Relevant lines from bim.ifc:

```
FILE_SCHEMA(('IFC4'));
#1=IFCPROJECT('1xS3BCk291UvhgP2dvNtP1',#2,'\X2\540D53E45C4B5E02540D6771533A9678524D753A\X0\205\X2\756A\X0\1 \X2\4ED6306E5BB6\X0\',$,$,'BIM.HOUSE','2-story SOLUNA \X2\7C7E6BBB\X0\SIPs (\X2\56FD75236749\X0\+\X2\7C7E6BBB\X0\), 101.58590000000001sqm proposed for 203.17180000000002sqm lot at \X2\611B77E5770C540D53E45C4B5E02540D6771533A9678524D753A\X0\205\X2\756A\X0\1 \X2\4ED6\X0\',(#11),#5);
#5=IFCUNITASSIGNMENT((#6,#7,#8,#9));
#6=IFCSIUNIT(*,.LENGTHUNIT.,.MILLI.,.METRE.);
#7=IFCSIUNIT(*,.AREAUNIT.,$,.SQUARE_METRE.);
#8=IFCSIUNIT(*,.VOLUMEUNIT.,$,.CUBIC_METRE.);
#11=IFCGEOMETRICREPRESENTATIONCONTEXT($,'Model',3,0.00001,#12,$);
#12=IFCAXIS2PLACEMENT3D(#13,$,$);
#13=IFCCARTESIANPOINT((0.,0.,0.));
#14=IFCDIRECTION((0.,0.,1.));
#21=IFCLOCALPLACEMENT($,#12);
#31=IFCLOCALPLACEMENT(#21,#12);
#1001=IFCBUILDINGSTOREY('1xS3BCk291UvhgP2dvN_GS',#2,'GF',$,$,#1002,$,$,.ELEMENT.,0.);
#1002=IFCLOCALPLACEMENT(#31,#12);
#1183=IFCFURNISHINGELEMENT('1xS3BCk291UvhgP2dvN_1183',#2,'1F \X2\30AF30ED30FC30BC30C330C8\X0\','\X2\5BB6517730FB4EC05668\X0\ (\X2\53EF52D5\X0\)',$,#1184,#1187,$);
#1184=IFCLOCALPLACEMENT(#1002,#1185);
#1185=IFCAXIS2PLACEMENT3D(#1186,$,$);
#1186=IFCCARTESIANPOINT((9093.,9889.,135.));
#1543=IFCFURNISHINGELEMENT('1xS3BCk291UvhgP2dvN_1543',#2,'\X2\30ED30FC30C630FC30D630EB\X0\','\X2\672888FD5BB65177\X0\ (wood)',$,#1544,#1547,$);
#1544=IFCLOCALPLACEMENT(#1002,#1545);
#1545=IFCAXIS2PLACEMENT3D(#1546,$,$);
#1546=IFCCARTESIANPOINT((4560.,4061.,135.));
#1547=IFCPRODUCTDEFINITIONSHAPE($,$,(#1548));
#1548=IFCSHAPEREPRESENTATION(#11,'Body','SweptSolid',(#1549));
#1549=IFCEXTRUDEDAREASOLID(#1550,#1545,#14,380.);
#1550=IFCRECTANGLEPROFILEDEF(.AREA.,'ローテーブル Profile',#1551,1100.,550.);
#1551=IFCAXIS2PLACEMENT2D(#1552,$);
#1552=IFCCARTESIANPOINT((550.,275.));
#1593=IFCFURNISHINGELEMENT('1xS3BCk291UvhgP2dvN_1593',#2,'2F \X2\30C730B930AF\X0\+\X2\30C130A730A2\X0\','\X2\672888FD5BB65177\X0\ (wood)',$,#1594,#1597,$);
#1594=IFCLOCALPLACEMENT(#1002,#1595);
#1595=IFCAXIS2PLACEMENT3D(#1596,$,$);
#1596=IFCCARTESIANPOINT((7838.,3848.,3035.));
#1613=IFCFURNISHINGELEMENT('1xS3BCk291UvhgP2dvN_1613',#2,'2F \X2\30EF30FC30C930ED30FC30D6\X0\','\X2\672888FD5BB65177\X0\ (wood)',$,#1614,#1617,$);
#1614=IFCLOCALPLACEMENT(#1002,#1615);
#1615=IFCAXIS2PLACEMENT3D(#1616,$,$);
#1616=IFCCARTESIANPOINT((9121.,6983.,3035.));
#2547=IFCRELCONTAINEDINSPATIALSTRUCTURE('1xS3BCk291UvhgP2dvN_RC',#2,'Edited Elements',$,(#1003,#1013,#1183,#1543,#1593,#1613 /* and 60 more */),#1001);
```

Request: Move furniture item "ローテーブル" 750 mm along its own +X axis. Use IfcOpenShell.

```python
import ifcopenshell
import ifcopenshell.api.geometry
import ifcopenshell.util.placement

model = ifcopenshell.open("bim.ifc")

item = model.by_guid("1xS3BCk291UvhgP2dvN_1543")
matrix = ifcopenshell.util.placement.get_local_placement(item.ObjectPlacement)
matrix[:3, 3] += matrix[:3, 0] * 750.0
ifcopenshell.api.geometry.edit_object_placement(model, product=item, matrix=matrix, is_si=False)

print(ifcopenshell.util.placement.get_local_placement(item.ObjectPlacement).round(3) + 0.0)

model.write("bim_edited.ifc")
```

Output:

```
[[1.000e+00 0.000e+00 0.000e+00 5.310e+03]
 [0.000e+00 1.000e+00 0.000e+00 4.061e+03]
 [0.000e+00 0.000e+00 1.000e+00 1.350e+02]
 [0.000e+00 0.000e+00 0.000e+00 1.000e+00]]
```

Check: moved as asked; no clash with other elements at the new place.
